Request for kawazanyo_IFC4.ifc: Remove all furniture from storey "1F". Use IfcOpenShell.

First a look at what the model holds.

```python
import ifcopenshell
import ifcopenshell.util.element

model = ifcopenshell.open("kawazanyo_IFC4.ifc")
print(model.schema)
storey = next(s for s in model.by_type("IfcBuildingStorey") if s.Name == "1F")
furniture = [e for e in ifcopenshell.util.element.get_decomposition(storey) if e.is_a("IfcFurnishingElement")]
seen = {}
for e in furniture:
    element_type = ifcopenshell.util.element.get_type(e)
    name = element_type.Name if element_type not in (None, e) else None
    seen[name] = seen.get(name, 0) + 1
for name, count in sorted(seen.items(), key=str):
    print(count, "x", name)
```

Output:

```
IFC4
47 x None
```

```python
import ifcopenshell
import ifcopenshell.api.root
import ifcopenshell.util.element

model = ifcopenshell.open("kawazanyo_IFC4.ifc")

storey = next(s for s in model.by_type("IfcBuildingStorey") if s.Name == "1F")
furniture = [e for e in ifcopenshell.util.element.get_decomposition(storey) if e.is_a("IfcFurnishingElement")]

for e in furniture:
    ifcopenshell.api.root.remove_product(model, product=e)
print(len(furniture), "removed")

model.write("kawazanyo_IFC4_v2.ifc")
```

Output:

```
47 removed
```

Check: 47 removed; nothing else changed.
